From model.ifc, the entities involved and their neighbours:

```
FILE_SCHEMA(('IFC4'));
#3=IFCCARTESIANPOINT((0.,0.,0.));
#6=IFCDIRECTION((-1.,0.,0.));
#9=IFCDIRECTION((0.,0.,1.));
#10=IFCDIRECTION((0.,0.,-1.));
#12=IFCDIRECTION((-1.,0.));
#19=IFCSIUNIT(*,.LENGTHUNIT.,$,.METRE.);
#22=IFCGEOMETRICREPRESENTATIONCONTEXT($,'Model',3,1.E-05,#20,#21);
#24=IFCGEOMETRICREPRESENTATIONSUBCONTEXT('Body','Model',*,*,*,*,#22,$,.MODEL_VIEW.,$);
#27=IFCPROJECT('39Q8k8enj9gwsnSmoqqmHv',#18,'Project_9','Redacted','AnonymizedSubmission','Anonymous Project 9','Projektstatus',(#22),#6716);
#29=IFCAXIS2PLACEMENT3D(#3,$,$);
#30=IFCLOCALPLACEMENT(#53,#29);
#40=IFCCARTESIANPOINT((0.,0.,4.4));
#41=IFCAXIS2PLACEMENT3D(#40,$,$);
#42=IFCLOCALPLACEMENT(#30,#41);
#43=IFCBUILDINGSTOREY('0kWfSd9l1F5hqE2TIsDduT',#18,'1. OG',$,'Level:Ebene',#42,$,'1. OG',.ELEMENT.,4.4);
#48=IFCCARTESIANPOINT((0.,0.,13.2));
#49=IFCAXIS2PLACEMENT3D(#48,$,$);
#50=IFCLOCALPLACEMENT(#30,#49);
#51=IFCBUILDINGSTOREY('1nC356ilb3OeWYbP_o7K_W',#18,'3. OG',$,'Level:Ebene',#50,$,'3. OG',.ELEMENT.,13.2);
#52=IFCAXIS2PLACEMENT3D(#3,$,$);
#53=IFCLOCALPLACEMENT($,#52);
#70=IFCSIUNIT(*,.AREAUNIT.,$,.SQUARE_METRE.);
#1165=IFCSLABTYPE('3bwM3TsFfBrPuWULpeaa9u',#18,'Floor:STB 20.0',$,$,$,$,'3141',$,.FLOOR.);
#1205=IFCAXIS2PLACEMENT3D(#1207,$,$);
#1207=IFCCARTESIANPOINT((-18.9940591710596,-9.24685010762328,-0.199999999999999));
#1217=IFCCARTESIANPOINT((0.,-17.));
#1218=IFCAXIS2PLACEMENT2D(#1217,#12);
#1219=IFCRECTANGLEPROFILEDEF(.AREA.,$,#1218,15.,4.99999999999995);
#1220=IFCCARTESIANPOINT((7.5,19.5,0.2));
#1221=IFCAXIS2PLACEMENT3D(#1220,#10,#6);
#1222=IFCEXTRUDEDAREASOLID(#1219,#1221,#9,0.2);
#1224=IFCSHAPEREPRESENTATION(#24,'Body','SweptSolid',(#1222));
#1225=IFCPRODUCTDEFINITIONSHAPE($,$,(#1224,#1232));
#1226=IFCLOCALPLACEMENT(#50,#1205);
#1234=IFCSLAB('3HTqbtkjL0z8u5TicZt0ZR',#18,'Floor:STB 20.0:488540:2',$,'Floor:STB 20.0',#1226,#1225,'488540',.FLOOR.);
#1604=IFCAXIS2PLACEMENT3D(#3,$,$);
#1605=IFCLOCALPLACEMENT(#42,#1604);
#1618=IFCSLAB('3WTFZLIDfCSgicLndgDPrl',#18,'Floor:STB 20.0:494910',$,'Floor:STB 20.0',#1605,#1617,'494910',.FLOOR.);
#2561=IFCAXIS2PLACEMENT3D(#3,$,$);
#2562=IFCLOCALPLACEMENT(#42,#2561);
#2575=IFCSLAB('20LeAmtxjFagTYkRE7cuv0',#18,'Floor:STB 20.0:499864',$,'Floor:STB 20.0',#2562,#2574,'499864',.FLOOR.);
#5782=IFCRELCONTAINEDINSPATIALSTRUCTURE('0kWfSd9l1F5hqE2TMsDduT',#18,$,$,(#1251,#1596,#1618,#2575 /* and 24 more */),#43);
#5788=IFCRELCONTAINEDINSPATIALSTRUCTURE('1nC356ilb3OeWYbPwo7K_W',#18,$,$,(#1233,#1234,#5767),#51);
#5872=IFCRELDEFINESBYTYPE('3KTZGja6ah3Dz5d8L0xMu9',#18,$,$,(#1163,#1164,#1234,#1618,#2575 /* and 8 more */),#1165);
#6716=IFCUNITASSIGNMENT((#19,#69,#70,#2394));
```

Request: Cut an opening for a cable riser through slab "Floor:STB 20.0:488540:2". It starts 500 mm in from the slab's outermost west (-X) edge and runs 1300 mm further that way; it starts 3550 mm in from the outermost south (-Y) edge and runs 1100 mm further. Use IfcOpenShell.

```python
import numpy as np
import ifcopenshell
import ifcopenshell.api.feature
import ifcopenshell.api.geometry
import ifcopenshell.api.root
import ifcopenshell.geom
import ifcopenshell.util.placement
import ifcopenshell.util.representation
import ifcopenshell.util.shape
import ifcopenshell.util.unit

model = ifcopenshell.open("model.ifc")
unit_scale = ifcopenshell.util.unit.calculate_unit_scale(model)
settings = ifcopenshell.geom.settings()


def volume(element):
    """Net volume in cubic metres, openings subtracted."""
    shape = ifcopenshell.geom.create_shape(settings, element)
    return ifcopenshell.util.shape.get_volume(shape.geometry)


slab = model.by_guid("3HTqbtkjL0z8u5TicZt0ZR")
before = volume(slab)

# Extent in the slab's own axes, in metres. The edges named are its -X and -Y sides.
slab_shape = ifcopenshell.geom.create_shape(settings, slab)
vertices = ifcopenshell.util.shape.get_vertices(slab_shape.geometry)
x_min, y_min, bottom = vertices.min(axis=0)
top = vertices[:, 2].max()

opening = ifcopenshell.api.root.create_entity(model, ifc_class="IfcOpeningElement", name="Cable riser opening", predefined_type="OPENING")
context = ifcopenshell.util.representation.get_context(model, "Model", "Body", "MODEL_VIEW")
width, depth = 1.3, 1.1
outline = [(0.0, 0.0), (width, 0.0), (width, depth), (0.0, depth), (0.0, 0.0)]
# Overshoot both faces by 50 mm so the cut is clean.
shape = ifcopenshell.api.geometry.add_slab_representation(
    model, context=context, depth=top - bottom + 0.1, polyline=outline
)
ifcopenshell.api.geometry.assign_representation(model, product=opening, representation=shape)

matrix = ifcopenshell.util.placement.get_local_placement(slab.ObjectPlacement)
matrix[:, 3] = matrix @ np.append(np.array([x_min + 0.5, y_min + 3.55, bottom - 0.05]) / unit_scale, 1.0)
ifcopenshell.api.geometry.edit_object_placement(model, product=opening, matrix=matrix, is_si=False)
ifcopenshell.api.feature.add_feature(model, feature=opening, element=slab)

after = volume(slab)

print(f"slab volume {before:.3f} -> {after:.3f} m3")

model.write("model-out.ifc")
```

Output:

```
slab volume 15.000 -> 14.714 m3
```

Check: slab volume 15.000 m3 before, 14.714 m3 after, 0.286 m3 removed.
